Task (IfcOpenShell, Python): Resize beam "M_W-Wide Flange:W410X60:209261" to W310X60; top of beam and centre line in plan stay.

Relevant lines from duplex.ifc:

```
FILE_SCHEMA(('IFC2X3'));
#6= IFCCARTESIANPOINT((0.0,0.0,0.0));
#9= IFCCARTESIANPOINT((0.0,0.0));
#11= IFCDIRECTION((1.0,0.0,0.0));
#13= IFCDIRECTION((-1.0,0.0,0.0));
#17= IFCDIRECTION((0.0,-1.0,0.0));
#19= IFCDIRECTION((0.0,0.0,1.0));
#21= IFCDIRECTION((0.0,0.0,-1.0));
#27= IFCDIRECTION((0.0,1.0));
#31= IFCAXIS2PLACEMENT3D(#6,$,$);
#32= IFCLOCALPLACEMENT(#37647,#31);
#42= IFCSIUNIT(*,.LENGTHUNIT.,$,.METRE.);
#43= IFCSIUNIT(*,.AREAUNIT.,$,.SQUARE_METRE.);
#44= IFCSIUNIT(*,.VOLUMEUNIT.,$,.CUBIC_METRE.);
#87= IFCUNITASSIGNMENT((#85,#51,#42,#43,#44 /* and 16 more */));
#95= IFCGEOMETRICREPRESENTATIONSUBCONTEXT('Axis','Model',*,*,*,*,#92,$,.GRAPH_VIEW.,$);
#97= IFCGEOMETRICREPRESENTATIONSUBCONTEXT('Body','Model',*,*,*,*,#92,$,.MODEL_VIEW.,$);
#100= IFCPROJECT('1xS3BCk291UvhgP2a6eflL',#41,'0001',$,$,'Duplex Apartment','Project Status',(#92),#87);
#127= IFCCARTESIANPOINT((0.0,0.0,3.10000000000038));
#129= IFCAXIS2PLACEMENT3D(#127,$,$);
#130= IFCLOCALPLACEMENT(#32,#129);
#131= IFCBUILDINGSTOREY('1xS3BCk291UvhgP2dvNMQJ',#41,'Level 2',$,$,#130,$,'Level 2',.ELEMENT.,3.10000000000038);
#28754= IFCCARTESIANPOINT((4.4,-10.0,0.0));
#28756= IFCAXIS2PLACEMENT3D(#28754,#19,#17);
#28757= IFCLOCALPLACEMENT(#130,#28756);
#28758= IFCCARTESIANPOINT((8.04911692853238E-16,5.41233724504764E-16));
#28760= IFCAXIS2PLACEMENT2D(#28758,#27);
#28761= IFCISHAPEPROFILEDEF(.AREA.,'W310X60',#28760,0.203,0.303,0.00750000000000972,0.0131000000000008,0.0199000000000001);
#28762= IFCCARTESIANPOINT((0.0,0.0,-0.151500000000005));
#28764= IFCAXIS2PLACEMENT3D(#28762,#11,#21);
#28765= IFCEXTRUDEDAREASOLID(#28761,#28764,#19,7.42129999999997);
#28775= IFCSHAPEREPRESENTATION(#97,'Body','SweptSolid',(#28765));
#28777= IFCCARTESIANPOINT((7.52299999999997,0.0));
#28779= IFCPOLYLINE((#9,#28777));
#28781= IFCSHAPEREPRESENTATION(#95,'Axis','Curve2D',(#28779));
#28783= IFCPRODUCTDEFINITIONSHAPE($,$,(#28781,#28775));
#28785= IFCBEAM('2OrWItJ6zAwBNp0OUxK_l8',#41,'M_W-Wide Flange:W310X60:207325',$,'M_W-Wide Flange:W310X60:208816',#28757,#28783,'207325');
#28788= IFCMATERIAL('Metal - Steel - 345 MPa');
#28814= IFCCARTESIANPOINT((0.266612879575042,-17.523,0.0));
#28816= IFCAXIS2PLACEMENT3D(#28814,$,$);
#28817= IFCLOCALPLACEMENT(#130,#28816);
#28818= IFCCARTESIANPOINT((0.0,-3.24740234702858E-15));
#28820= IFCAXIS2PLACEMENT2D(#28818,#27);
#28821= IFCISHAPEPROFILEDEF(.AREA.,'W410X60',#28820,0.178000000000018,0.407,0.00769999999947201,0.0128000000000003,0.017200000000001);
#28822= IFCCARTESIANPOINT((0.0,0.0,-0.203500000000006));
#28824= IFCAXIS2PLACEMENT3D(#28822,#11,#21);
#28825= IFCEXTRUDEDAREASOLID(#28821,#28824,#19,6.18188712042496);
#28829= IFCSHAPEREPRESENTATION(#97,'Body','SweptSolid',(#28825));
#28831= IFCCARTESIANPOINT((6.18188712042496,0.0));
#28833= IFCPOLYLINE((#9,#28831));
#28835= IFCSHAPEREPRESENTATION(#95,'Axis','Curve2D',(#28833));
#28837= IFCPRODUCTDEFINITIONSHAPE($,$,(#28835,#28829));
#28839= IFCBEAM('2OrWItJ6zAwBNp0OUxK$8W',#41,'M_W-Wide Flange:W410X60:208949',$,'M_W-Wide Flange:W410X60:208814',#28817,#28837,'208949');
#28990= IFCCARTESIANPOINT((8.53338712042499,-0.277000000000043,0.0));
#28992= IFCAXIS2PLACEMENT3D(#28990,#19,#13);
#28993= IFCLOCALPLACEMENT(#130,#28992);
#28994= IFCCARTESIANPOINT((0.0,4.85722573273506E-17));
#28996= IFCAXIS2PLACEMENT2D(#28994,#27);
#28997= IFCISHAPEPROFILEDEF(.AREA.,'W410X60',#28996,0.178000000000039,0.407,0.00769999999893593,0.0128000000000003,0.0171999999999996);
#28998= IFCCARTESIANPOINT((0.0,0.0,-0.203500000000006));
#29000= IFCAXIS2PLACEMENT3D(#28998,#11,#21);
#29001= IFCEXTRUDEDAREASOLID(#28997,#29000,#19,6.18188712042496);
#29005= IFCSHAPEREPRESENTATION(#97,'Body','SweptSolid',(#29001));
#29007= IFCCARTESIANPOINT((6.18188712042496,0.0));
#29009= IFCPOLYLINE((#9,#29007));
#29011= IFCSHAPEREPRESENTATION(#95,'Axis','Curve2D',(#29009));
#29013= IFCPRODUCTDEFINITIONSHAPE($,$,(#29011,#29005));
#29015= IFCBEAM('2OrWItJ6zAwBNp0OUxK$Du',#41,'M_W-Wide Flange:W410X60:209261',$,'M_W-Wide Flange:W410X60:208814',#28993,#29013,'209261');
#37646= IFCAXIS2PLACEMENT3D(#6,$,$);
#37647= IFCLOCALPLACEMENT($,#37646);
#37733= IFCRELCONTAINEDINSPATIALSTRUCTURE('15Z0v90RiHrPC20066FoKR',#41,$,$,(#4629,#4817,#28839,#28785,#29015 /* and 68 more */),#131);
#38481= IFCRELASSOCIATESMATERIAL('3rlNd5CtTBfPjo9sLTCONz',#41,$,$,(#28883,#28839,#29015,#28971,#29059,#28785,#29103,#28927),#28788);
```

```python
import ifcopenshell
import ifcopenshell.util.element
import ifcopenshell.util.representation

model = ifcopenshell.open("duplex.ifc")

member = model.by_guid("2OrWItJ6zAwBNp0OUxK$Du")
source = next(p for p in model.by_type("IfcIShapeProfileDef") if p.ProfileName == "W310X60")

body = ifcopenshell.util.representation.get_representation(member, "Model", "Body")
solid = body.Items[0]
old_profile = solid.SweptArea

# Copy the section's sizes but keep this member's own profile position.
profile = ifcopenshell.util.element.copy(model, source)
# Profiles are centred, so shift by half the change in depth to hold the top.
shift = (old_profile.OverallDepth - profile.OverallDepth) / 2
x, y = old_profile.Position.Location.Coordinates
up = (-1.0, 0.0)  # upwards, in the solid's own plane
location = model.createIfcCartesianPoint((x + up[0] * shift, y + up[1] * shift))
profile.Position = model.createIfcAxis2Placement2D(location, old_profile.Position.RefDirection)
solid.SweptArea = profile
if not model.get_total_inverses(old_profile):
    ifcopenshell.util.element.remove_deep2(model, old_profile)
member.Name = member.Name.replace("W410X60", "W310X60")
member.ObjectType = member.ObjectType.replace("W410X60", "W310X60")

print(solid.SweptArea)

model.write("duplex_rev.ifc")
```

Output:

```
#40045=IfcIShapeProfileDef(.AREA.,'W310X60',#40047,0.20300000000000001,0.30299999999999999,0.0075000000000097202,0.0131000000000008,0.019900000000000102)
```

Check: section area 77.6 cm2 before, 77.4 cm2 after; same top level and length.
